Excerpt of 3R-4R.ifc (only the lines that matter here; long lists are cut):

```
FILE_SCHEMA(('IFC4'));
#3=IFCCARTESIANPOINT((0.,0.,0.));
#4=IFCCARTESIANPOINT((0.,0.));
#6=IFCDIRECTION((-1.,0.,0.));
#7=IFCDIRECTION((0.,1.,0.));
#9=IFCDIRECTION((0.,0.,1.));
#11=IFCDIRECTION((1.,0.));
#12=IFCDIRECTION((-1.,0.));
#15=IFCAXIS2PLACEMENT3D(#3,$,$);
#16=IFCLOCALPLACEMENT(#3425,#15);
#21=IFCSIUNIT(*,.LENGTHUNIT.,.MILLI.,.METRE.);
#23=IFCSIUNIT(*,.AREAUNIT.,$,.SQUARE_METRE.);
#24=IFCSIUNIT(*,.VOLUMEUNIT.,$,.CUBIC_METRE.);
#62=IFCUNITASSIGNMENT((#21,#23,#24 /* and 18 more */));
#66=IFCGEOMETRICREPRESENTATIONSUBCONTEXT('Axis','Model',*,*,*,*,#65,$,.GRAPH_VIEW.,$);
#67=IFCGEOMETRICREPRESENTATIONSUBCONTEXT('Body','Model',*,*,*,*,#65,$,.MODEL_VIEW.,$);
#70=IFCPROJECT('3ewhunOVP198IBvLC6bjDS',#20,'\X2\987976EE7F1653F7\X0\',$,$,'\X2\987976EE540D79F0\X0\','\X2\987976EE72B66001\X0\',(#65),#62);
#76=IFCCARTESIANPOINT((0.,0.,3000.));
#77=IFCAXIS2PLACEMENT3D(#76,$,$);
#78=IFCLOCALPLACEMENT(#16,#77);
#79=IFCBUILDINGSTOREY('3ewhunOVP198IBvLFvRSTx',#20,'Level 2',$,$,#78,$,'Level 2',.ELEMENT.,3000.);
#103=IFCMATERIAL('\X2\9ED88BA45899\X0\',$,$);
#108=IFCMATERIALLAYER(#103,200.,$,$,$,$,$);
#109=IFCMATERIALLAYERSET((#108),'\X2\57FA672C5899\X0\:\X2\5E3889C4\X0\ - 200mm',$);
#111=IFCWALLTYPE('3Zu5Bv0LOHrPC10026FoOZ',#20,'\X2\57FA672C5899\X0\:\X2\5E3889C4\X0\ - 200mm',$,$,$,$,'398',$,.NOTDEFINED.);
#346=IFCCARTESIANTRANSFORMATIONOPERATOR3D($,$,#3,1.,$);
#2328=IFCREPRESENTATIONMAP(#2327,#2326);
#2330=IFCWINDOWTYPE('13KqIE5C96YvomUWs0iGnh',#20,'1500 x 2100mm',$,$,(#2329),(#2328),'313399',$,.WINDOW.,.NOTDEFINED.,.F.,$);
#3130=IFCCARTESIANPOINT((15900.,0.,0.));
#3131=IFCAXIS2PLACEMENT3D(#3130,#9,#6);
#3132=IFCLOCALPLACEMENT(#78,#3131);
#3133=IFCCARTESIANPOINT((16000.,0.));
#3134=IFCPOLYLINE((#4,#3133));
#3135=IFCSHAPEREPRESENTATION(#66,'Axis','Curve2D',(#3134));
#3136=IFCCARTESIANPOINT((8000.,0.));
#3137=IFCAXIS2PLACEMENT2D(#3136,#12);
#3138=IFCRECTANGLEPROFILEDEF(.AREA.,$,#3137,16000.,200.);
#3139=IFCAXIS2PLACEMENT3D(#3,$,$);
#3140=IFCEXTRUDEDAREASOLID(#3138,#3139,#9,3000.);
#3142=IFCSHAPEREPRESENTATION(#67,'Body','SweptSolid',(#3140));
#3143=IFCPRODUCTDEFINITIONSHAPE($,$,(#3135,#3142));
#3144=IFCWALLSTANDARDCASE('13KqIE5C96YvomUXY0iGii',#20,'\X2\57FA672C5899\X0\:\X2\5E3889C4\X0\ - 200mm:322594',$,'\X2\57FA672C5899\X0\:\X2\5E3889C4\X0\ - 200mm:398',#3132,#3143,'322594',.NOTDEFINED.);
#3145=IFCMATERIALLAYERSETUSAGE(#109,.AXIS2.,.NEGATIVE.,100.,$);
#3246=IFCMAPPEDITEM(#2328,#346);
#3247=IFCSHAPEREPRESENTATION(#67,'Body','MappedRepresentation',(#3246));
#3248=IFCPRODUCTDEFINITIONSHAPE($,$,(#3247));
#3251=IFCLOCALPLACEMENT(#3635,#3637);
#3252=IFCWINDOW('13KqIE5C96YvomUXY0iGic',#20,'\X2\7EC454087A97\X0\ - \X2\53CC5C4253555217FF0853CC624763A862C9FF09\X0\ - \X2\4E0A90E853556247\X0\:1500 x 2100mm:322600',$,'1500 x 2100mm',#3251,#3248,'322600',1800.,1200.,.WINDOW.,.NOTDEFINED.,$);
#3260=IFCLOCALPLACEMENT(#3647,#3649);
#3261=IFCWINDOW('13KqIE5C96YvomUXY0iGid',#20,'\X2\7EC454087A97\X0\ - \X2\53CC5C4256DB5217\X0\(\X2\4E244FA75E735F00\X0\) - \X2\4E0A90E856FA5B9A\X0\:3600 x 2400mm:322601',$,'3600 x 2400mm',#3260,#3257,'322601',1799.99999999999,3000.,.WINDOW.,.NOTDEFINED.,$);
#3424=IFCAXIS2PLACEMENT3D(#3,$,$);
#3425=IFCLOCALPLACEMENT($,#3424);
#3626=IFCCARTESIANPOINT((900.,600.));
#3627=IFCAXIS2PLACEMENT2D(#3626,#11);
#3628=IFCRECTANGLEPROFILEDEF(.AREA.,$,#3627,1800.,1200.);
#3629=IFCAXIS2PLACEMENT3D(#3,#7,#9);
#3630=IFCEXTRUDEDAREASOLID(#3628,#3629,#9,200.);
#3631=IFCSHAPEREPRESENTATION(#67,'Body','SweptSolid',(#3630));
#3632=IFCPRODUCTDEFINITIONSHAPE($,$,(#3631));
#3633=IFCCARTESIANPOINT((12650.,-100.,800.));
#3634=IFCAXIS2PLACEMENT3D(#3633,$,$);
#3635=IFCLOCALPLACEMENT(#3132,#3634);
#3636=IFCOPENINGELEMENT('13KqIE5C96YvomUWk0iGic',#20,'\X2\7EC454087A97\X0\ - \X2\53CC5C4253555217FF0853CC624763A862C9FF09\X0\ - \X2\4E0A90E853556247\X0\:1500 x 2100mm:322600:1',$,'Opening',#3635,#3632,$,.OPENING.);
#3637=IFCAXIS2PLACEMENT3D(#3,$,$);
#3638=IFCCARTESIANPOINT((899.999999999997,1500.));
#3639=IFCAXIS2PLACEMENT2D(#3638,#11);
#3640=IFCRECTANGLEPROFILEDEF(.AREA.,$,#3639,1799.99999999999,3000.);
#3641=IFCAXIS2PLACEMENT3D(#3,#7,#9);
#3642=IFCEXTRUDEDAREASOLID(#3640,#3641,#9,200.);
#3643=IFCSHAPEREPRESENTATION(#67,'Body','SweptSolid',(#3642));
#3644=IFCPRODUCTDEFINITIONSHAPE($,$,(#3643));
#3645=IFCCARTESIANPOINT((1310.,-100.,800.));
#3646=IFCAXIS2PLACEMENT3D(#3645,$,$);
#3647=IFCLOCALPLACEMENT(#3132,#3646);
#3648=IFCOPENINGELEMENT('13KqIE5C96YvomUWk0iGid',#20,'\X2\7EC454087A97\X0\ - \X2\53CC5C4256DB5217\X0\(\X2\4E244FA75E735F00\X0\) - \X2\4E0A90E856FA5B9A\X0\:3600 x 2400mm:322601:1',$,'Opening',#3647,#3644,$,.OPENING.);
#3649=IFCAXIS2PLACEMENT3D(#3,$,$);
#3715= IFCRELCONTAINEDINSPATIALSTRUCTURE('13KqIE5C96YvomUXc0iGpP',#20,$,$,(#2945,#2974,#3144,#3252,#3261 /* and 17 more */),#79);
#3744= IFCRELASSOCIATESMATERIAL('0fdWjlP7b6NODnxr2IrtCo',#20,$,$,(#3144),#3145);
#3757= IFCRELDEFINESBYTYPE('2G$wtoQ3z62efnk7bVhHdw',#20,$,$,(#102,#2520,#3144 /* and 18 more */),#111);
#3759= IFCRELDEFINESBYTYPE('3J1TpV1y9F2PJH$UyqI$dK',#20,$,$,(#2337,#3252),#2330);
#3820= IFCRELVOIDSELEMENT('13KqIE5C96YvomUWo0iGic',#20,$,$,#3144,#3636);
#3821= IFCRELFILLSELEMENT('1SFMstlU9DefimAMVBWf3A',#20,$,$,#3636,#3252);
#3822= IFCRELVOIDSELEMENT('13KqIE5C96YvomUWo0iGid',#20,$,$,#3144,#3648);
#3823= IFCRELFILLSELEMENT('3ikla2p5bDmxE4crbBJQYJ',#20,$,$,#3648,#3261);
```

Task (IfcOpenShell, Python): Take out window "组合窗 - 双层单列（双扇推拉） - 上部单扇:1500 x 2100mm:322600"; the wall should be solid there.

```python
import ifcopenshell
import ifcopenshell.api.feature
import ifcopenshell.api.root
import ifcopenshell.geom
import ifcopenshell.util.shape

model = ifcopenshell.open("3R-4R.ifc")
settings = ifcopenshell.geom.settings()


def volume(element):
    """Net volume in cubic metres, openings subtracted."""
    shape = ifcopenshell.geom.create_shape(settings, element)
    return ifcopenshell.util.shape.get_volume(shape.geometry)


window = model.by_guid("13KqIE5C96YvomUXY0iGic")
opening = window.FillsVoids[0].RelatingOpeningElement
wall = opening.VoidsElements[0].RelatingBuildingElement
before = volume(wall)

ifcopenshell.api.root.remove_product(model, product=window)
ifcopenshell.api.feature.remove_feature(model, feature=opening)

after = volume(wall)

print(f"wall volume {before:.3f} -> {after:.3f} m3")

model.write("3R-4R_v2.ifc")
```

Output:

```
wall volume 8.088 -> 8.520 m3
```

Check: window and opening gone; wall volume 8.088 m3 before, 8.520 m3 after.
